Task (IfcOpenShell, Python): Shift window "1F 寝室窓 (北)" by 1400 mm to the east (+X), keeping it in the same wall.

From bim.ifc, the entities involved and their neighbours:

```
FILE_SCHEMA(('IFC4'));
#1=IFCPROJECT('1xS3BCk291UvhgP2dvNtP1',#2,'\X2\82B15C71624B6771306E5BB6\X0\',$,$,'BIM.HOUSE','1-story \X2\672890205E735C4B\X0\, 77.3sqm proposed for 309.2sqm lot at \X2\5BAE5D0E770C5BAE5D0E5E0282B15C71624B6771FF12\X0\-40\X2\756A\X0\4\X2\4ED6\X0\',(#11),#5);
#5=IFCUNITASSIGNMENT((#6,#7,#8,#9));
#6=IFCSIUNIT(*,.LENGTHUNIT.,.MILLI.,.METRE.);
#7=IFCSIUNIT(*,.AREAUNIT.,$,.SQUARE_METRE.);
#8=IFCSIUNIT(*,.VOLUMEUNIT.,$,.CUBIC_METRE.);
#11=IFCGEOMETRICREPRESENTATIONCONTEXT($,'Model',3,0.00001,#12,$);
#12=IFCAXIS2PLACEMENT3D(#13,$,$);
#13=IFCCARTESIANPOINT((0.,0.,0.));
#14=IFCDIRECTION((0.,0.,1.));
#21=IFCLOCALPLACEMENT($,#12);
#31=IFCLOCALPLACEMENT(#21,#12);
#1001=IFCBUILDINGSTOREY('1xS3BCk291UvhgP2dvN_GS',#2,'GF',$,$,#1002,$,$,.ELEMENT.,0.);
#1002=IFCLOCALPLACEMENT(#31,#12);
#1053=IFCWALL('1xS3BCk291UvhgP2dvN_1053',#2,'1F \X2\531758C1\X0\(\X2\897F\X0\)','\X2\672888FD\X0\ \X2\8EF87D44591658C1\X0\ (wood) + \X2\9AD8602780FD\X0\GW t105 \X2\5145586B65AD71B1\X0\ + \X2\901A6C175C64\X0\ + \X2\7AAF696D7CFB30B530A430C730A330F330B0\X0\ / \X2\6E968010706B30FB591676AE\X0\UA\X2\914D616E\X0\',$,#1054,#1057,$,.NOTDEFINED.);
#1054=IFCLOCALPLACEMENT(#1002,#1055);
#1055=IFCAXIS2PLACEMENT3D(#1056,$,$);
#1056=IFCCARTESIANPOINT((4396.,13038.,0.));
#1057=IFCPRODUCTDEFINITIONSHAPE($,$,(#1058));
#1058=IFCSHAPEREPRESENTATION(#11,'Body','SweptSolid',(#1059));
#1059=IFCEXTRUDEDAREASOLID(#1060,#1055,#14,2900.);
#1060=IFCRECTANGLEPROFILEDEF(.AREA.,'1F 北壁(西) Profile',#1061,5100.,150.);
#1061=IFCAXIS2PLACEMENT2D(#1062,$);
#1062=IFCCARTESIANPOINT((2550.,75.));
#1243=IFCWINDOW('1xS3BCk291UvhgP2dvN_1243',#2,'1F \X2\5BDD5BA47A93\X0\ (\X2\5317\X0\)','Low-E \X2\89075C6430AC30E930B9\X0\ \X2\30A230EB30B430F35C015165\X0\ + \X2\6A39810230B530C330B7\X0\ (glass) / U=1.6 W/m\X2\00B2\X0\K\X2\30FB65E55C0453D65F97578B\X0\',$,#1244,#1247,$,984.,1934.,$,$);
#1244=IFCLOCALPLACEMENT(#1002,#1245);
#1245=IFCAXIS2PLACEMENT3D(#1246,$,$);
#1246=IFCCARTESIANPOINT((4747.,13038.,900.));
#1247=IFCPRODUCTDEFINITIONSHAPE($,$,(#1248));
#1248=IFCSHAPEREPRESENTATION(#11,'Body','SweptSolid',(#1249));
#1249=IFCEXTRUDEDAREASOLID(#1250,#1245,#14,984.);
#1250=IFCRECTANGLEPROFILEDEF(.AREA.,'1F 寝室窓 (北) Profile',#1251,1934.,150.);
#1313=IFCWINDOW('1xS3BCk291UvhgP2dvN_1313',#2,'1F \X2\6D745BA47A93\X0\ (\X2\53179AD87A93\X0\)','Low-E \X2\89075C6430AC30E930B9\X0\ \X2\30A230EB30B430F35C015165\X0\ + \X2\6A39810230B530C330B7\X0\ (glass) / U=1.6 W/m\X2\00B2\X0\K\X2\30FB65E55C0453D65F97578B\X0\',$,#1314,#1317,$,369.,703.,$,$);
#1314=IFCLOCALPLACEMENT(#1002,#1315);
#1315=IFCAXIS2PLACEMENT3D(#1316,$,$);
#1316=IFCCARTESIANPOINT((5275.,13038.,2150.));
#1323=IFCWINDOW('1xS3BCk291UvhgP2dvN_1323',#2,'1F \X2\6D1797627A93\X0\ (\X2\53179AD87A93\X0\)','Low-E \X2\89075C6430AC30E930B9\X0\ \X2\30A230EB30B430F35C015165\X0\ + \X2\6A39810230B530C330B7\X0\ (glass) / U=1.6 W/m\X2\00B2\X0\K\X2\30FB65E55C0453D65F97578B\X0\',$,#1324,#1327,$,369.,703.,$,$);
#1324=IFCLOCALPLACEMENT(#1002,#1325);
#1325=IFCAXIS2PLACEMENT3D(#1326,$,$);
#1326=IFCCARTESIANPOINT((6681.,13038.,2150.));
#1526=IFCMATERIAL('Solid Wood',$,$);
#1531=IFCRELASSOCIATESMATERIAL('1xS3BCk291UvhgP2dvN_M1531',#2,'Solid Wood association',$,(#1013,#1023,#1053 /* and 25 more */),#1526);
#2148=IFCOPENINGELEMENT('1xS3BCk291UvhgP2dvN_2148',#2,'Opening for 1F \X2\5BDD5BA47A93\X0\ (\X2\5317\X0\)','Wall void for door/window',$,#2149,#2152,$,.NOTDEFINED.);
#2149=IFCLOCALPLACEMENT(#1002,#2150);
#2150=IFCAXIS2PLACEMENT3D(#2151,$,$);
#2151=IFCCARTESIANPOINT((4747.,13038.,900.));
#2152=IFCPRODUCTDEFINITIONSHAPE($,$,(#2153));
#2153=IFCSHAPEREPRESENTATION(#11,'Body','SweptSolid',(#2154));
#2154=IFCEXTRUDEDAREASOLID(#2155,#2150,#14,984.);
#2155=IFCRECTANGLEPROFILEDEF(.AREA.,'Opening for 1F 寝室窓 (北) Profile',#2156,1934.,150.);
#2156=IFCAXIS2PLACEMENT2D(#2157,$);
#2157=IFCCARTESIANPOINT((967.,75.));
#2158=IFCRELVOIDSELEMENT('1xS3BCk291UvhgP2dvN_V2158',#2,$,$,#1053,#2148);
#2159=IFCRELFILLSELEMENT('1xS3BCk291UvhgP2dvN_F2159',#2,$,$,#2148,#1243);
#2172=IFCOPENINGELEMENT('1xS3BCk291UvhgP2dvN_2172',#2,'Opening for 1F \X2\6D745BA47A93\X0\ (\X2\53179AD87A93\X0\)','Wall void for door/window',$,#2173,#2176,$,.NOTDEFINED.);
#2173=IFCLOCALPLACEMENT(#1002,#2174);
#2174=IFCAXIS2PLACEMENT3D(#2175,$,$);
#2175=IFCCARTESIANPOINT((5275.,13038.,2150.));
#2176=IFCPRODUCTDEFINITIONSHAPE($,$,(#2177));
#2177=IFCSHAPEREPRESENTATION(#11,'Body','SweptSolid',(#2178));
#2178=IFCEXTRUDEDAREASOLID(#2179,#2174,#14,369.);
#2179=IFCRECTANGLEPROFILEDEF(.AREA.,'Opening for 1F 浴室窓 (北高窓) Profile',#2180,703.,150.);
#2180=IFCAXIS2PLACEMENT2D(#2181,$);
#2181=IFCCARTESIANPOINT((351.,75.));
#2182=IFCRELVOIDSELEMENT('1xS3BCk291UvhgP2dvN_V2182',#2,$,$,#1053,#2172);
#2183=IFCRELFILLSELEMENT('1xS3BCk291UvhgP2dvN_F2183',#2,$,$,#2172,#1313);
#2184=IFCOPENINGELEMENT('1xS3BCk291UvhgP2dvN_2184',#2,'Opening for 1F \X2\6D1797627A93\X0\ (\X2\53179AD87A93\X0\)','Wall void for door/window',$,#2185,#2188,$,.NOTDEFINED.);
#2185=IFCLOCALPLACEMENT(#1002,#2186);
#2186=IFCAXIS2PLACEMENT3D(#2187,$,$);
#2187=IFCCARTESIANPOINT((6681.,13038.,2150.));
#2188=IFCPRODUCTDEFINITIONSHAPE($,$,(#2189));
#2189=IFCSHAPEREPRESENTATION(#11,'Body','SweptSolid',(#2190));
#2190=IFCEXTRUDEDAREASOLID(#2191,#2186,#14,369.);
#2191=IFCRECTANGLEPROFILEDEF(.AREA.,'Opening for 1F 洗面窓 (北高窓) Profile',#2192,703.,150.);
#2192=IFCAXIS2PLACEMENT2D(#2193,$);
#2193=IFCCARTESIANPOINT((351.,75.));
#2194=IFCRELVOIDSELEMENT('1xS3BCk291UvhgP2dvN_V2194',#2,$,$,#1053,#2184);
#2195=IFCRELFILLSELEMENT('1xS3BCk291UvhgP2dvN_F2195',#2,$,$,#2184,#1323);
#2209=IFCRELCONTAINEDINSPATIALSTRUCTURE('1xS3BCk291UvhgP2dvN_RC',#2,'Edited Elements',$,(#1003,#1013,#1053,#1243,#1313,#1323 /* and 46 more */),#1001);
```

```python
import ifcopenshell
import ifcopenshell.api.geometry
import ifcopenshell.util.placement
import ifcopenshell.util.unit

model = ifcopenshell.open("bim.ifc")
unit_scale = ifcopenshell.util.unit.calculate_unit_scale(model)

window = model.by_guid("1xS3BCk291UvhgP2dvN_1243")
opening = window.FillsVoids[0].RelatingOpeningElement
wall = opening.VoidsElements[0].RelatingBuildingElement

wall_matrix = ifcopenshell.util.placement.get_local_placement(wall.ObjectPlacement)
shift = wall_matrix[:3, 0] * 1.4 / unit_scale
before = ifcopenshell.util.placement.get_local_placement(window.ObjectPlacement)[:3, 3].copy()

# The window is not placed relative to its opening, so move both.
for product in (opening, window):
    matrix = ifcopenshell.util.placement.get_local_placement(product.ObjectPlacement)
    matrix[:3, 3] += shift
    ifcopenshell.api.geometry.edit_object_placement(model, product=product, matrix=matrix, is_si=False)

after = ifcopenshell.util.placement.get_local_placement(window.ObjectPlacement)[:3, 3]
print("window moved by", (after - before).round(3) + 0.0)

model.write("bim_updated.ifc")
```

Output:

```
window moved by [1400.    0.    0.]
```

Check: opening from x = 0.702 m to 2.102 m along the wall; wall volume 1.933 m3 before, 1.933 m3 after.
